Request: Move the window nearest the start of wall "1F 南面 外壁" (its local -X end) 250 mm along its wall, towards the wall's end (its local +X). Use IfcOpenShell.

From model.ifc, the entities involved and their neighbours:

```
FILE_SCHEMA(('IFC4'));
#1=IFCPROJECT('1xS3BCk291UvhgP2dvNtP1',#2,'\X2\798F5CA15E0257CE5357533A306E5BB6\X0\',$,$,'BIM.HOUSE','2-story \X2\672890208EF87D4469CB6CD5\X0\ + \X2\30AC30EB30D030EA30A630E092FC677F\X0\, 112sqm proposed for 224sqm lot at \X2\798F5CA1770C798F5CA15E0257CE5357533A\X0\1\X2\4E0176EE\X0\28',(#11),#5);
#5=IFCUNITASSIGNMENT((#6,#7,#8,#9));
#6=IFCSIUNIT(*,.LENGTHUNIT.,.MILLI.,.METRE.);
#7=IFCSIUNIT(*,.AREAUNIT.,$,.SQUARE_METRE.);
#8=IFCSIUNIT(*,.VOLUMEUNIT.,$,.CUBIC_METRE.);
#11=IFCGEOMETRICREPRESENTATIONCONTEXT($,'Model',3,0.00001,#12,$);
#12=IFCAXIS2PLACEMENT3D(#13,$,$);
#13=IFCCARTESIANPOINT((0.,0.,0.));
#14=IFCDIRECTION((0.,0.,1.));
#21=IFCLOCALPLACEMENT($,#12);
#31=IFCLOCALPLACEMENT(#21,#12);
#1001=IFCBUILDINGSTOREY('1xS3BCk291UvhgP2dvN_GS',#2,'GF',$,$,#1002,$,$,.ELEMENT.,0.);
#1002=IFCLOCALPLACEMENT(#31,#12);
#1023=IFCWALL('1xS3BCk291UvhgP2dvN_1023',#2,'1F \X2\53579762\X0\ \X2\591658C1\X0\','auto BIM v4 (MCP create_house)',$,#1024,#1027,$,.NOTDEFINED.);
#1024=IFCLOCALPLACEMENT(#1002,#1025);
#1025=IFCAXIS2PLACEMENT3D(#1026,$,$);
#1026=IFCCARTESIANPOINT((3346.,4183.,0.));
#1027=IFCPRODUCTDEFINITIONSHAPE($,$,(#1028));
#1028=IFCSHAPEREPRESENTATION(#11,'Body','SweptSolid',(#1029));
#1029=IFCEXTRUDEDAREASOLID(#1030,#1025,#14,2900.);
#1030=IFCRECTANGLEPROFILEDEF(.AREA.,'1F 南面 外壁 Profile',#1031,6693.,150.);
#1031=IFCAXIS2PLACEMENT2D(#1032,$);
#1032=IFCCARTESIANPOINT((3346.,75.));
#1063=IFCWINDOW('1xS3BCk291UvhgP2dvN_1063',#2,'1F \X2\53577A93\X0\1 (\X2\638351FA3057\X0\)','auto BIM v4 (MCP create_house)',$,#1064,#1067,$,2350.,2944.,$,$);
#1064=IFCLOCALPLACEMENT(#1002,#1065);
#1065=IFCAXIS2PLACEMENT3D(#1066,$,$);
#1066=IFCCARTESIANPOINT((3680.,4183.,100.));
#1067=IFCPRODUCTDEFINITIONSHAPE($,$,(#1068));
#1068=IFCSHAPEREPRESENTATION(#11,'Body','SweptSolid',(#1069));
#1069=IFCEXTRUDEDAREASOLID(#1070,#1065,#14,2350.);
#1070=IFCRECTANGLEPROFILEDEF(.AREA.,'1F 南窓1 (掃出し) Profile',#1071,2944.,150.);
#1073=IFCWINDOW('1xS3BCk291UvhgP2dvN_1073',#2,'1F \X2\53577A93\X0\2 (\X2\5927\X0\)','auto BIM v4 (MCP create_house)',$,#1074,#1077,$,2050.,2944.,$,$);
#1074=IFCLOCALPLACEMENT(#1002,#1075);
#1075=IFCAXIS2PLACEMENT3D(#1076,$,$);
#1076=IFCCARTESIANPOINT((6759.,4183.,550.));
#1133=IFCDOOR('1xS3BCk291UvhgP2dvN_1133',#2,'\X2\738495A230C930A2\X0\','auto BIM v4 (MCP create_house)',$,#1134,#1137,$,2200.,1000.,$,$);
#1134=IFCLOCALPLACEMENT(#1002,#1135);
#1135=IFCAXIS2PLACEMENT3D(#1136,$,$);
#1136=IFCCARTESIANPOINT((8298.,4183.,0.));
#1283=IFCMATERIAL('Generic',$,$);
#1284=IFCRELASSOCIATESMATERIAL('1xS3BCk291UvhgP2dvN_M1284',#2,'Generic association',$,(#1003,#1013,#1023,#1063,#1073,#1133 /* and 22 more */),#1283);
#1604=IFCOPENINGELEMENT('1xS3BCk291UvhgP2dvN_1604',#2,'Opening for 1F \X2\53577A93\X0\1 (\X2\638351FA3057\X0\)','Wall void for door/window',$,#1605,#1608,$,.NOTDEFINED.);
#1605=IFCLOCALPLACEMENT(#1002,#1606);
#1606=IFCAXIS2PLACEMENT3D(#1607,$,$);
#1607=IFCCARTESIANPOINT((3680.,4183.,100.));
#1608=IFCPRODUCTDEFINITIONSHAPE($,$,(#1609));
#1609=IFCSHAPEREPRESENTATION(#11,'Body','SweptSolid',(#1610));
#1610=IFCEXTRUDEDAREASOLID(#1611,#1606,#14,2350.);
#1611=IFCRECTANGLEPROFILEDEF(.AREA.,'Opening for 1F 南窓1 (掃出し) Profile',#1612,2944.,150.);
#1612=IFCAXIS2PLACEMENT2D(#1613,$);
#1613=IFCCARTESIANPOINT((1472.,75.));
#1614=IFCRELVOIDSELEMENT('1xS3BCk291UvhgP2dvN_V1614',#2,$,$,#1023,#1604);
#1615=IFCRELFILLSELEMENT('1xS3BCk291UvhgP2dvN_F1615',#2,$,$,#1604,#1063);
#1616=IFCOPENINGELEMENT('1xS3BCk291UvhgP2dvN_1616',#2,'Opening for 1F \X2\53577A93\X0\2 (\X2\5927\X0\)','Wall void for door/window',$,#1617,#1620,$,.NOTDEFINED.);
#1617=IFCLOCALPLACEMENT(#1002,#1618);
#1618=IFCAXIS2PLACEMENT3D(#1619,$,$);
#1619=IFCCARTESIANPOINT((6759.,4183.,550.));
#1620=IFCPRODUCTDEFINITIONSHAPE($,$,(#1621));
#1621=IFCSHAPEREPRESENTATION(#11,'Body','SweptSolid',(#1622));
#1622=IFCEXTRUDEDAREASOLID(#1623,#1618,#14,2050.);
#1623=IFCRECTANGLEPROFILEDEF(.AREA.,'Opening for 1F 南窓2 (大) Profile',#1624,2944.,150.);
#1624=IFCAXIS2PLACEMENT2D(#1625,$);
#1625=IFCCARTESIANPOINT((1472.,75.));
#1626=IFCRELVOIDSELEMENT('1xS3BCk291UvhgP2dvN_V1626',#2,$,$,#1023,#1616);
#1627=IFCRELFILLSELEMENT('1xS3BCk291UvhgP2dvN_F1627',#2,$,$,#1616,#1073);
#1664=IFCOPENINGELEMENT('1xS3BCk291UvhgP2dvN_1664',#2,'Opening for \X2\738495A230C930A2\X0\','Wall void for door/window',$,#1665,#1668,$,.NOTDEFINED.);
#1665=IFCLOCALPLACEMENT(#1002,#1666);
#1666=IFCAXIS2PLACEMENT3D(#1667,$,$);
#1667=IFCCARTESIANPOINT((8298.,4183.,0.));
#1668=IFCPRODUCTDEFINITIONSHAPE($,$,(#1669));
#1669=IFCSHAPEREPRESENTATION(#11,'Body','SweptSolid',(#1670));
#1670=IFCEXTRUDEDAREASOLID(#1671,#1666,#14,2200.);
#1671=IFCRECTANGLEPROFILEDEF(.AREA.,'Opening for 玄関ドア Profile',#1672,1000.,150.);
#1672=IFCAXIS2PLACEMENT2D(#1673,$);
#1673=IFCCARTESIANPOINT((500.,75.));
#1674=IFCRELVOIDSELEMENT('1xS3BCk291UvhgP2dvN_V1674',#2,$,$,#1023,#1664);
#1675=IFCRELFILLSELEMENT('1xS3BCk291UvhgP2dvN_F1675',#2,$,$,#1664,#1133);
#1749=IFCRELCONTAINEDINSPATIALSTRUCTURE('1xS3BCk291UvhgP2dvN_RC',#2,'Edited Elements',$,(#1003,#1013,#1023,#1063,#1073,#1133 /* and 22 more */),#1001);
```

```python
import ifcopenshell
import ifcopenshell.api.geometry
import ifcopenshell.util.placement

model = ifcopenshell.open("model.ifc")

window = model.by_id(1063)
opening = window.FillsVoids[0].RelatingOpeningElement
wall = opening.VoidsElements[0].RelatingBuildingElement

wall_matrix = ifcopenshell.util.placement.get_local_placement(wall.ObjectPlacement)
shift = wall_matrix[:3, 0] * 250.0
before = ifcopenshell.util.placement.get_local_placement(window.ObjectPlacement)[:3, 3].copy()

# The window is not placed relative to its opening, so move both.
for product in (opening, window):
    matrix = ifcopenshell.util.placement.get_local_placement(product.ObjectPlacement)
    matrix[:3, 3] += shift
    ifcopenshell.api.geometry.edit_object_placement(model, product=product, matrix=matrix, is_si=False)

after = ifcopenshell.util.placement.get_local_placement(window.ObjectPlacement)[:3, 3]
print("window moved by", (after - before).round(3) + 0.0)

model.write("model_v2.ifc")
```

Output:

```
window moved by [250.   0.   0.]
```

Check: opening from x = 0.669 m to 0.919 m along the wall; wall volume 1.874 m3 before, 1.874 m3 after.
